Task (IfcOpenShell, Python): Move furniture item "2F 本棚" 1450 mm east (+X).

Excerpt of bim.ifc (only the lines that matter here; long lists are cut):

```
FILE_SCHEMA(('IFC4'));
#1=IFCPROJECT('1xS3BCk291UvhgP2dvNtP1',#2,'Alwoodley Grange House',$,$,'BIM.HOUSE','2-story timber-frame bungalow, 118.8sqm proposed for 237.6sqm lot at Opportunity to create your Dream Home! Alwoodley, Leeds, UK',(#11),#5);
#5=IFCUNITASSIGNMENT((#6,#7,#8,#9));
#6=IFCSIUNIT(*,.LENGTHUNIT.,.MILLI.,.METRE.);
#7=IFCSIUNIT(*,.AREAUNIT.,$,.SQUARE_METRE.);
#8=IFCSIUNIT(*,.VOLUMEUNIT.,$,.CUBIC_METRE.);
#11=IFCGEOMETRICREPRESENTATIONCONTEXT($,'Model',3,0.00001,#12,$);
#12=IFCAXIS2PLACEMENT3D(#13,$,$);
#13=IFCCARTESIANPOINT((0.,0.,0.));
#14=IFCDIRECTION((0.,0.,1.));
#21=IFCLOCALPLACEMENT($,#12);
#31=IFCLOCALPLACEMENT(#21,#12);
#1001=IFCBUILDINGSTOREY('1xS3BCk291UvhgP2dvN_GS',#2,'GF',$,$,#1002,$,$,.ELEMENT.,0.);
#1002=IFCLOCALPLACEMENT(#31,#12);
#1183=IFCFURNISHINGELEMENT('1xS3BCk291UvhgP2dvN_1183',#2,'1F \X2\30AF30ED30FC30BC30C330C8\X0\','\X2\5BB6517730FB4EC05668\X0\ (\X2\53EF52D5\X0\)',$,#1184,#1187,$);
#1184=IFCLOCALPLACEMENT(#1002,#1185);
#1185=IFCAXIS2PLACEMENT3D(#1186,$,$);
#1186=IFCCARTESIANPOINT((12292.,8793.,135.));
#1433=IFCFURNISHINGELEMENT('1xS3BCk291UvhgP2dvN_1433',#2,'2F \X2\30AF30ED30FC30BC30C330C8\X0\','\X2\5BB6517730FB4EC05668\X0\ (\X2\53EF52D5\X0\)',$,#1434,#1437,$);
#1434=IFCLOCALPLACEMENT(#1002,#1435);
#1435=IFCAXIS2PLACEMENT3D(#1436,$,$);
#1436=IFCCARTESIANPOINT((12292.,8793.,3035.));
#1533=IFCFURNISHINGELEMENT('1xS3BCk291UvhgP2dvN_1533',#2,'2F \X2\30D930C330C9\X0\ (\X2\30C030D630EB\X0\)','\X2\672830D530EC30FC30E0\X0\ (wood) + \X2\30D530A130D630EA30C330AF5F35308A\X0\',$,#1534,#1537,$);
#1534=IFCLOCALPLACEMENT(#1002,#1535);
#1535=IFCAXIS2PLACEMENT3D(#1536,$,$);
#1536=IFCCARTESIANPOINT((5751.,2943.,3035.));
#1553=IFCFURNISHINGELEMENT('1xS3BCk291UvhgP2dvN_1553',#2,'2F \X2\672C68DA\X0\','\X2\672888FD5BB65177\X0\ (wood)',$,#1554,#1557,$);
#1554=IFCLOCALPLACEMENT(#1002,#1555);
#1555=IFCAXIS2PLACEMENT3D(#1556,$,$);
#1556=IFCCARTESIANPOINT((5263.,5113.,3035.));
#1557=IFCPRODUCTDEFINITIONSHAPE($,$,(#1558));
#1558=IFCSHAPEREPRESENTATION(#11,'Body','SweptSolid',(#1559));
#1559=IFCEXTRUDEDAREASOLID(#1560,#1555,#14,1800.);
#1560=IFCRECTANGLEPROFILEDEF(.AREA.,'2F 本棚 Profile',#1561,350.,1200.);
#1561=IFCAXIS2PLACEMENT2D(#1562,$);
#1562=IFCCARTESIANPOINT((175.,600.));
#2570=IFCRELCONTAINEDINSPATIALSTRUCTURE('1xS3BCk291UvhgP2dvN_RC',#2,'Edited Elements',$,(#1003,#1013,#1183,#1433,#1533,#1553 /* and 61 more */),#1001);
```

```python
import ifcopenshell
import ifcopenshell.api.geometry
import ifcopenshell.util.placement
import ifcopenshell.util.unit

model = ifcopenshell.open("bim.ifc")
unit_scale = ifcopenshell.util.unit.calculate_unit_scale(model)

item = model.by_guid("1xS3BCk291UvhgP2dvN_1553")
matrix = ifcopenshell.util.placement.get_local_placement(item.ObjectPlacement)
matrix[0, 3] += 1.45 / unit_scale
ifcopenshell.api.geometry.edit_object_placement(model, product=item, matrix=matrix, is_si=False)

print(ifcopenshell.util.placement.get_local_placement(item.ObjectPlacement).round(3) + 0.0)

model.write("bim-out.ifc")
```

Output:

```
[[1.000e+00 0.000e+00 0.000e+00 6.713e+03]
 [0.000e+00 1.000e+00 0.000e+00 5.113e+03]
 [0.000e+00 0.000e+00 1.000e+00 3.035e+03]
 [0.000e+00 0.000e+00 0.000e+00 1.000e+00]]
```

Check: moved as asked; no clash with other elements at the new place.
